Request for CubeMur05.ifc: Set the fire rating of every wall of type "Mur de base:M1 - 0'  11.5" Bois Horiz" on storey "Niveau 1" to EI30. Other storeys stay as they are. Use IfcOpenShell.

First a look at what the model holds.

```python
import ifcopenshell
import ifcopenshell.util.element

model = ifcopenshell.open("CubeMur05.ifc")
print(model.schema)
storey = next(s for s in model.by_type("IfcBuildingStorey") if s.Name == "Niveau 1")
walls = [e for e in ifcopenshell.util.element.get_decomposition(storey) if e.is_a("IfcWall")]
seen = {}
for e in walls:
    element_type = ifcopenshell.util.element.get_type(e)
    key = (element_type.Name if element_type != e and element_type else None, ifcopenshell.util.element.get_pset(e, "Pset_WallCommon", "FireRating"))
    seen[key] = seen.get(key, 0) + 1
for (name, value), count in sorted(seen.items(), key=str):
    print(count, "x", name, "|", value)
```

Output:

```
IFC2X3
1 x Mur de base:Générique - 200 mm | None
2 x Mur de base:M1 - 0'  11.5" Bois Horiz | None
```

```python
import ifcopenshell
import ifcopenshell.api.pset
import ifcopenshell.util.element

model = ifcopenshell.open("CubeMur05.ifc")

storey = next(s for s in model.by_type("IfcBuildingStorey") if s.Name == "Niveau 1")
walls = [e for e in ifcopenshell.util.element.get_decomposition(storey) if e.is_a("IfcWall")]

count = 0
for e in walls:
    element_type = ifcopenshell.util.element.get_type(e)
    if element_type in (None, e) or element_type.Name != 'Mur de base:M1 - 0\'  11.5" Bois Horiz':
        continue
    # add_pset returns the element's existing set when there is one.
    pset = ifcopenshell.api.pset.add_pset(model, product=e, name="Pset_WallCommon")
    ifcopenshell.api.pset.edit_pset(model, pset=pset, properties={"FireRating": "EI30"})
    count += 1

print(count, "walls updated")

model.write("CubeMur05-out.ifc")
```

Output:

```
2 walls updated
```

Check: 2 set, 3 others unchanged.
